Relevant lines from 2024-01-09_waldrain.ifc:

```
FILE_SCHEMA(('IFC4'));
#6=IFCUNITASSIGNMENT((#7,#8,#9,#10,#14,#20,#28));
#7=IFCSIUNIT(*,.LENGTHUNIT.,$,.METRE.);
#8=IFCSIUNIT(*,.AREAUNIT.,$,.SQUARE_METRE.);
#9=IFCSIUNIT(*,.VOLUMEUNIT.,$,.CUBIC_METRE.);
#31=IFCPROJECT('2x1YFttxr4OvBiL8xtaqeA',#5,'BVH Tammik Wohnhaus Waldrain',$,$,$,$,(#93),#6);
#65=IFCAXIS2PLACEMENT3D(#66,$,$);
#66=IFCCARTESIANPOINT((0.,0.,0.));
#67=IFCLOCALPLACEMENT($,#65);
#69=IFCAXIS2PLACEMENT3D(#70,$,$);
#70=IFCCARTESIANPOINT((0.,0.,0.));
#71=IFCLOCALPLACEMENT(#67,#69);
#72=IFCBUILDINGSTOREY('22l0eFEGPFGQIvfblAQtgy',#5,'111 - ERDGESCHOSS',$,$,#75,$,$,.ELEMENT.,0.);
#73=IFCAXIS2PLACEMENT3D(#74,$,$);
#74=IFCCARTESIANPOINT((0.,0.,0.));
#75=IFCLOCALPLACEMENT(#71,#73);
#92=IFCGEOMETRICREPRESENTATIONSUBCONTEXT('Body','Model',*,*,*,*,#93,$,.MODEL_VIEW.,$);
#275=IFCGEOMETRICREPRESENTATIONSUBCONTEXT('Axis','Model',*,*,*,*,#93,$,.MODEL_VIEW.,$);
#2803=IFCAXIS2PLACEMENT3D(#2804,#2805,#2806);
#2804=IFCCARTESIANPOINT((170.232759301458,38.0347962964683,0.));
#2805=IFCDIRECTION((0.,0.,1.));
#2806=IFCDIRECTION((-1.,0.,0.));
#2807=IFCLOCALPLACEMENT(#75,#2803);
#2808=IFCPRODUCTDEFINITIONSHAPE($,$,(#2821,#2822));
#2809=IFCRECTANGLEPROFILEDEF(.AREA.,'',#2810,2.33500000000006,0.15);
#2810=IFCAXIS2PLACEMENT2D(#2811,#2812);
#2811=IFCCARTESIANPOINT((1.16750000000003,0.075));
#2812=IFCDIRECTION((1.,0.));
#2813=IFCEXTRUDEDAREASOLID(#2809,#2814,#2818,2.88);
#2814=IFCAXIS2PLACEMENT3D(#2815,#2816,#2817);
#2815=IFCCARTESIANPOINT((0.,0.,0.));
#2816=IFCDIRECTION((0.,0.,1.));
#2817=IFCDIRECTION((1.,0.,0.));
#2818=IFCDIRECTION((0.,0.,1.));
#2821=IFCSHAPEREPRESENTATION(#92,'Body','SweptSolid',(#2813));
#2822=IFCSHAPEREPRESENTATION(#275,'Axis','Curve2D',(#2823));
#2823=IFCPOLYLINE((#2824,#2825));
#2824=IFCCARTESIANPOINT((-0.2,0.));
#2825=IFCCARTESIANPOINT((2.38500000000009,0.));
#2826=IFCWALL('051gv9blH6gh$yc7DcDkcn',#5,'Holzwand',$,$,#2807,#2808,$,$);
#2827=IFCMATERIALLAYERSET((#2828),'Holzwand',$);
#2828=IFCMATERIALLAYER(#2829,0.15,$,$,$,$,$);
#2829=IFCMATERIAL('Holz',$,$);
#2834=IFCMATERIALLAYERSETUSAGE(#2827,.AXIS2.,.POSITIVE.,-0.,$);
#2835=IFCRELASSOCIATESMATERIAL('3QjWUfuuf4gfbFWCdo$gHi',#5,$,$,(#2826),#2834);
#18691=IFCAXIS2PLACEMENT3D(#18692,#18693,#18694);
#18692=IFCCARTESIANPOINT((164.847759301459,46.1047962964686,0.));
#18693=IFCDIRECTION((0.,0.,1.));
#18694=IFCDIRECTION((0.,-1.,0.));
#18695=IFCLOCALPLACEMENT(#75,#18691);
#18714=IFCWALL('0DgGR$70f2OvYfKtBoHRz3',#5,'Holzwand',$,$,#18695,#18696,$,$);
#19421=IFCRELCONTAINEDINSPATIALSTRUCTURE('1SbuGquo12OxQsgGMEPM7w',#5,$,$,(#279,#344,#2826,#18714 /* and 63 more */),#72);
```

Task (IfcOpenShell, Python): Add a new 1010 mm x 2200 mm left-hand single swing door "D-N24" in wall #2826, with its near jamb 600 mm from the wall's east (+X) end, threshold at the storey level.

```python
import numpy as np
import ifcopenshell
import ifcopenshell.api.feature
import ifcopenshell.api.geometry
import ifcopenshell.api.root
import ifcopenshell.api.spatial
import ifcopenshell.geom
import ifcopenshell.util.element
import ifcopenshell.util.placement
import ifcopenshell.util.representation
import ifcopenshell.util.shape
import ifcopenshell.util.unit

model = ifcopenshell.open("2024-01-09_waldrain.ifc")
unit_scale = ifcopenshell.util.unit.calculate_unit_scale(model)
settings = ifcopenshell.geom.settings()


def volume(element):
    """Net volume in cubic metres, openings subtracted."""
    shape = ifcopenshell.geom.create_shape(settings, element)
    return ifcopenshell.util.shape.get_volume(shape.geometry)


wall = model.by_guid("051gv9blH6gh$yc7DcDkcn")
storey = ifcopenshell.util.element.get_container(wall, ifc_class="IfcBuildingStorey")
context = ifcopenshell.util.representation.get_context(model, "Model", "Body", "MODEL_VIEW")
before = volume(wall)

width, height, from_end, sill = 1.01, 2.2, 0.6, 0.0  # metres

# The wall runs along its own X axis, and the end named is its -X end.
wall_shape = ifcopenshell.geom.create_shape(settings, wall)
x, y, z = ifcopenshell.util.shape.get_vertices(wall_shape.geometry).T
start = x.min() + from_end
face, thickness = float(y.min()), float(y.max() - y.min())
wall_matrix = ifcopenshell.util.placement.get_local_placement(wall.ObjectPlacement)
level = ifcopenshell.util.placement.get_local_placement(storey.ObjectPlacement)[2, 3]


def in_wall(x, y):
    """Placement at x, y metres in the wall's axes, at sill height."""
    matrix = wall_matrix.copy()
    matrix[:, 3] = wall_matrix @ np.array([x / unit_scale, y / unit_scale, 0.0, 1.0])
    matrix[2, 3] = level + sill / unit_scale
    return matrix


# Opening: a box that overshoots both wall faces by 50 mm.
opening = ifcopenshell.api.root.create_entity(model, ifc_class="IfcOpeningElement", predefined_type="OPENING")
box = ifcopenshell.api.geometry.add_wall_representation(
    model, context=context, length=width, height=height, thickness=thickness + 0.1
)
ifcopenshell.api.geometry.assign_representation(model, product=opening, representation=box)
ifcopenshell.api.geometry.edit_object_placement(model, product=opening, matrix=in_wall(start, face - 0.05), is_si=False)
ifcopenshell.api.feature.add_feature(model, feature=opening, element=wall)

door = ifcopenshell.api.root.create_entity(model, ifc_class="IfcDoor", name="D-N24", predefined_type="DOOR")
door.OverallWidth, door.OverallHeight = width / unit_scale, height / unit_scale
door.OperationType = "SINGLE_SWING_LEFT"
body = ifcopenshell.api.geometry.add_door_representation(
    model,
    context=context,
    overall_width=door.OverallWidth,
    overall_height=door.OverallHeight,
    operation_type="SINGLE_SWING_LEFT",
    lining_properties={"LiningDepth": thickness / unit_scale, "ThresholdDepth": thickness / unit_scale},
)
ifcopenshell.api.geometry.assign_representation(model, product=door, representation=body)
ifcopenshell.api.spatial.assign_container(model, products=[door], relating_structure=storey)
ifcopenshell.api.feature.add_filling(model, opening=opening, element=door)

# The lining spans the wall, so the door starts at the wall face.
ifcopenshell.api.geometry.edit_object_placement(model, product=door, matrix=in_wall(start, face), is_si=False)

after = volume(wall)

print(f"wall volume {before:.3f} -> {after:.3f} m3")

model.write("2024-01-09_waldrain_edited.ifc")
```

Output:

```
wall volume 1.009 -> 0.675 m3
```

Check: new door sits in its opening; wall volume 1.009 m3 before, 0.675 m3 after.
